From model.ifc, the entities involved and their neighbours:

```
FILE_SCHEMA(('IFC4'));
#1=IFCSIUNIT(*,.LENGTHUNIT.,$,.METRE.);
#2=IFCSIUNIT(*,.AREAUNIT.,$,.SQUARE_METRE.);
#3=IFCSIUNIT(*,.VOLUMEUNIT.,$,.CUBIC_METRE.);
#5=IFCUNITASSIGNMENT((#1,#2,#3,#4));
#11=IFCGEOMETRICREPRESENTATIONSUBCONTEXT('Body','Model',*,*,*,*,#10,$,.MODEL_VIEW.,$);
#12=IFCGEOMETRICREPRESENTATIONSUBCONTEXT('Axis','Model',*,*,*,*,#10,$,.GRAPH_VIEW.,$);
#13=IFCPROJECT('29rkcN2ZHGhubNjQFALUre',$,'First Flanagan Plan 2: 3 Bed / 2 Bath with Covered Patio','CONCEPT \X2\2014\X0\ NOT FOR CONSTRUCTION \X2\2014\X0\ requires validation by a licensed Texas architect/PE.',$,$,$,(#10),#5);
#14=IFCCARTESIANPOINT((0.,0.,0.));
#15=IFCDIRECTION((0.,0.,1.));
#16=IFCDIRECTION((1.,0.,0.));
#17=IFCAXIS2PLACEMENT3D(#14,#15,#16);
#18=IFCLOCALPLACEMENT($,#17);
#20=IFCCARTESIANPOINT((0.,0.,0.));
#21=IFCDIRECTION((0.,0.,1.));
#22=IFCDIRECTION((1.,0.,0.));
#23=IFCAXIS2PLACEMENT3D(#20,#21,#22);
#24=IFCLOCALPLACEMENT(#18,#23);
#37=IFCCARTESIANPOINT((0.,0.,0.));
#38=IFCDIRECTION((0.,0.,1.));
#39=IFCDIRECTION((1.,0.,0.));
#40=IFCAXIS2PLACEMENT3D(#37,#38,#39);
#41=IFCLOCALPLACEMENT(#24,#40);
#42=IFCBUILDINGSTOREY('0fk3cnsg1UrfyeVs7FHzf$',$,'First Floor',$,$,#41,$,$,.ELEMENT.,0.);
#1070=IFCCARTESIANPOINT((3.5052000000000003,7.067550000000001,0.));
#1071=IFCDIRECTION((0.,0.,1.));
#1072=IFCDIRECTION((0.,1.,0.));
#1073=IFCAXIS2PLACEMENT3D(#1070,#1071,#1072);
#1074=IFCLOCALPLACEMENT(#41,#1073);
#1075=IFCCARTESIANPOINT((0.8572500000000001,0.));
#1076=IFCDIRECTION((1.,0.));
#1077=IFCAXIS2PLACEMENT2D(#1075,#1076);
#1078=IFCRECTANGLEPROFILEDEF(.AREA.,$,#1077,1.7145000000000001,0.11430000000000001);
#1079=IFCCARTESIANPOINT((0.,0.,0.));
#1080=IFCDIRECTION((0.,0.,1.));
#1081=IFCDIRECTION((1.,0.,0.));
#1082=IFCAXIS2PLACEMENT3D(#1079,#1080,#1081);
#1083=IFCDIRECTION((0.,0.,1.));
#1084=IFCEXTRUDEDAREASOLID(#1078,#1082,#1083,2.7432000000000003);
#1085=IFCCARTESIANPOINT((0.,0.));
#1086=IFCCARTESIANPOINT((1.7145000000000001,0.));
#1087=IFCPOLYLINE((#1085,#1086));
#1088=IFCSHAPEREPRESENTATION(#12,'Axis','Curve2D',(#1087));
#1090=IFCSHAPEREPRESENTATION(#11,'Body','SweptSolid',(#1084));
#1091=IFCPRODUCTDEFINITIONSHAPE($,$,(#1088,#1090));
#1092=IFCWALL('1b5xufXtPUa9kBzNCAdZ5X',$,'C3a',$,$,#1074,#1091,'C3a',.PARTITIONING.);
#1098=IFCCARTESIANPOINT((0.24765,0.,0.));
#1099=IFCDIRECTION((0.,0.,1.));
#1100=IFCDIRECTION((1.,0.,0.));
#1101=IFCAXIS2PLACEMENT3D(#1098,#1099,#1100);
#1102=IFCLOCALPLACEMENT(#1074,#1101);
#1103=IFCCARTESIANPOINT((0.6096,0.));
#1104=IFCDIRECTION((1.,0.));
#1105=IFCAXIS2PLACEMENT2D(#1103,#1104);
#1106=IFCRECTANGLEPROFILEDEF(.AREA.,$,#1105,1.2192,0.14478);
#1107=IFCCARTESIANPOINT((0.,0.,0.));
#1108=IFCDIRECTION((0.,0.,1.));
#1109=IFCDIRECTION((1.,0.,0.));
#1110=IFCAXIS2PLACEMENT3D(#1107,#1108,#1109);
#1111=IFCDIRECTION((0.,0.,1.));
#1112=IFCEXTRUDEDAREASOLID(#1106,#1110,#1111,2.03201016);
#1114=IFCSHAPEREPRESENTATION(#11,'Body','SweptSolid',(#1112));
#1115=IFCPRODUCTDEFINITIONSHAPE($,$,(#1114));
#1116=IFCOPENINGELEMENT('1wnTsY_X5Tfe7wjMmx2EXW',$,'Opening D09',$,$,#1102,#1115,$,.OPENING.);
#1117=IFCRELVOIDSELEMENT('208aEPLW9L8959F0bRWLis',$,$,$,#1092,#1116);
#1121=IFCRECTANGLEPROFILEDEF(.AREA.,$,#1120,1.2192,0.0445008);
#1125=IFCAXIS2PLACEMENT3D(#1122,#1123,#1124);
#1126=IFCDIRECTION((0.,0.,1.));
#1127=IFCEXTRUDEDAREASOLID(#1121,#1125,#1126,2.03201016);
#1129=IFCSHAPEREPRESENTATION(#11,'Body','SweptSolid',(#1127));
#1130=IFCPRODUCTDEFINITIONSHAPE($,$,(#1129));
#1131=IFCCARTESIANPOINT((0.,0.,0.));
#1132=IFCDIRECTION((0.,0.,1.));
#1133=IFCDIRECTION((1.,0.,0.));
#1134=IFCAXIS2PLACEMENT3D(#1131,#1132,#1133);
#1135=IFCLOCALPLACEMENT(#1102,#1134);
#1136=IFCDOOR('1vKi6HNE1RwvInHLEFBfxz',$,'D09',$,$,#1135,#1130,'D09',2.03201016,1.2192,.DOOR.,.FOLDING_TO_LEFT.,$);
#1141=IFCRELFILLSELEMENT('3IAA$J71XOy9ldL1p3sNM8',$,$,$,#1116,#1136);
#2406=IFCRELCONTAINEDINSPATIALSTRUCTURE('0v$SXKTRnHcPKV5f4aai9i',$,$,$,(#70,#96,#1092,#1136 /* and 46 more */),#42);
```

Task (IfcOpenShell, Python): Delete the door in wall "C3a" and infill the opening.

```python
import ifcopenshell
import ifcopenshell.api.feature
import ifcopenshell.api.root
import ifcopenshell.geom
import ifcopenshell.util.shape

model = ifcopenshell.open("model.ifc")
settings = ifcopenshell.geom.settings()


def volume(element):
    """Net volume in cubic metres, openings subtracted."""
    shape = ifcopenshell.geom.create_shape(settings, element)
    return ifcopenshell.util.shape.get_volume(shape.geometry)


door = model.by_guid("1vKi6HNE1RwvInHLEFBfxz")
opening = door.FillsVoids[0].RelatingOpeningElement
wall = opening.VoidsElements[0].RelatingBuildingElement
before = volume(wall)

ifcopenshell.api.root.remove_product(model, product=door)
ifcopenshell.api.feature.remove_feature(model, feature=opening)

after = volume(wall)

print(f"wall volume {before:.3f} -> {after:.3f} m3")

model.write("model_edited.ifc")
```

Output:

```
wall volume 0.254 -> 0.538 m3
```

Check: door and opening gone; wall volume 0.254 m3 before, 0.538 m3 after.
